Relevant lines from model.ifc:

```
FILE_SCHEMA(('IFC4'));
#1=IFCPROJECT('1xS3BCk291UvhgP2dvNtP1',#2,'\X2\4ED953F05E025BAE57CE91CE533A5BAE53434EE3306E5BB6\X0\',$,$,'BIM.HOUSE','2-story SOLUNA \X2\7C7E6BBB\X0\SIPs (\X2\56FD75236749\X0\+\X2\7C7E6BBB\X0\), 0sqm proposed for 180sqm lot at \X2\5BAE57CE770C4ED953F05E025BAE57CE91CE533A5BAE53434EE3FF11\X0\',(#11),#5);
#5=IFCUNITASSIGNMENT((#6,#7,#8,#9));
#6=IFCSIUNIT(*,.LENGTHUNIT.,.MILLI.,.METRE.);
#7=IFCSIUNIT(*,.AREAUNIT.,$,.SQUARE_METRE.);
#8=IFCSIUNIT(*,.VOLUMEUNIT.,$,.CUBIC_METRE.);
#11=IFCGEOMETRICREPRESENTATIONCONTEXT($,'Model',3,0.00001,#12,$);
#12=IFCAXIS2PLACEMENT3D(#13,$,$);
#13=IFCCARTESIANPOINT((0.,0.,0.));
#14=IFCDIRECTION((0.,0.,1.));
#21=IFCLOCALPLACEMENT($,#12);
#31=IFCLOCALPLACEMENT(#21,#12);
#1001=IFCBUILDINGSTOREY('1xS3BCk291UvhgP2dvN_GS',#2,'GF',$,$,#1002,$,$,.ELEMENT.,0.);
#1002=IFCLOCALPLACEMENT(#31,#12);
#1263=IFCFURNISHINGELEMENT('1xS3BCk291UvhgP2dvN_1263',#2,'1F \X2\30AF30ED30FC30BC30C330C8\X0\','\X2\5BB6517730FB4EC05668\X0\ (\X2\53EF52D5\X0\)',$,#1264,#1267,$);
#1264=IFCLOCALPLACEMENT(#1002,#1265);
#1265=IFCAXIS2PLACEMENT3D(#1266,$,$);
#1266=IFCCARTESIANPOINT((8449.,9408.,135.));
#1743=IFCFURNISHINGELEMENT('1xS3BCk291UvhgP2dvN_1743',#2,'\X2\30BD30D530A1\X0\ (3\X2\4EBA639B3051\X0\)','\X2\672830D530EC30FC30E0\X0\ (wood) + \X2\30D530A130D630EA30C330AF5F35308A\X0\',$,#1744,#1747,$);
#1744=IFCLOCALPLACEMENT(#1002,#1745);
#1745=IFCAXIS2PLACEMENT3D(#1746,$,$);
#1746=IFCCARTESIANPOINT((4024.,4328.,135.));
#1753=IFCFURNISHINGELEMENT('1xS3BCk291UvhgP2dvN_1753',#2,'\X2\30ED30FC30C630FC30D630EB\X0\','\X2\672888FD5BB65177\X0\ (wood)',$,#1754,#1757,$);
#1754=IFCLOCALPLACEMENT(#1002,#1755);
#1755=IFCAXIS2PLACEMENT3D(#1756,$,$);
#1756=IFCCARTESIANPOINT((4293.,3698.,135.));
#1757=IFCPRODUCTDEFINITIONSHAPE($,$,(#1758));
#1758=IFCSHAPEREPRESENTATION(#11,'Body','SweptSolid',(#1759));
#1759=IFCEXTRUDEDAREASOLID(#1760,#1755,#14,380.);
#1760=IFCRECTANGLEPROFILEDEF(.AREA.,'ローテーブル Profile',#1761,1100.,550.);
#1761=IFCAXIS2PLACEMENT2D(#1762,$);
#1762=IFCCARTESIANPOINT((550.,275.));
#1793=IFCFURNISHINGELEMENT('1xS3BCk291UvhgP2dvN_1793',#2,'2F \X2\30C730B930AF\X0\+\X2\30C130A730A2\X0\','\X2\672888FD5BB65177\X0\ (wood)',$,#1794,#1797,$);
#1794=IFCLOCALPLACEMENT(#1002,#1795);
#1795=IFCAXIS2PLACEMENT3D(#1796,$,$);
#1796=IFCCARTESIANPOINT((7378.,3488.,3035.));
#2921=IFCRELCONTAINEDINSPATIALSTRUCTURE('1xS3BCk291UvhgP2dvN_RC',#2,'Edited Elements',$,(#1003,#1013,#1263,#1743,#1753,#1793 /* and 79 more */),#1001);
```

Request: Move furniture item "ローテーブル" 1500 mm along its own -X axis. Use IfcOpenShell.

```python
import ifcopenshell
import ifcopenshell.api.geometry
import ifcopenshell.util.placement

model = ifcopenshell.open("model.ifc")

item = model.by_id(1753)
matrix = ifcopenshell.util.placement.get_local_placement(item.ObjectPlacement)
matrix[:3, 3] -= matrix[:3, 0] * 1500.0
ifcopenshell.api.geometry.edit_object_placement(model, product=item, matrix=matrix, is_si=False)

print(ifcopenshell.util.placement.get_local_placement(item.ObjectPlacement).round(3) + 0.0)

model.write("model_v2.ifc")
```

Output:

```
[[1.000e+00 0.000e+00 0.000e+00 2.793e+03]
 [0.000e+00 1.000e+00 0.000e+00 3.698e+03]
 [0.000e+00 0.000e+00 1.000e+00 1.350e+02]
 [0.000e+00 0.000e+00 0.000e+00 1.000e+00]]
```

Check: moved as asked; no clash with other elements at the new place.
